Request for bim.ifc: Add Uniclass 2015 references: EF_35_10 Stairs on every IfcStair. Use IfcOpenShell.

First a look at what the model holds.

```python
import ifcopenshell

model = ifcopenshell.open("bim.ifc")
print(model.schema)
print("classifications:", [c.Name for c in model.by_type("IfcClassification")])
for ifc_class in ("IfcDoor", "IfcRoof", "IfcStair", "IfcWall", "IfcWindow"):
    print(ifc_class, len(model.by_type(ifc_class)))
```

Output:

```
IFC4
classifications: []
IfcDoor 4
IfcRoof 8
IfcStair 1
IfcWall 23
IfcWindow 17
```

```python
import ifcopenshell
import ifcopenshell.api.classification

model = ifcopenshell.open("bim.ifc")

system = ifcopenshell.api.classification.add_classification(model, classification="Uniclass 2015")

codes = {
    "IfcStair": ("EF_35_10", "Stairs"),
}
for ifc_class, (code, name) in codes.items():
    products = model.by_type(ifc_class)
    ifcopenshell.api.classification.add_reference(
        model, products=products, classification=system, identification=code, name=name
    )
    print(code, len(products))

model.write("bim_edited.ifc")
```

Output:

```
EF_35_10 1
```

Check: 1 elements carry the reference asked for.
